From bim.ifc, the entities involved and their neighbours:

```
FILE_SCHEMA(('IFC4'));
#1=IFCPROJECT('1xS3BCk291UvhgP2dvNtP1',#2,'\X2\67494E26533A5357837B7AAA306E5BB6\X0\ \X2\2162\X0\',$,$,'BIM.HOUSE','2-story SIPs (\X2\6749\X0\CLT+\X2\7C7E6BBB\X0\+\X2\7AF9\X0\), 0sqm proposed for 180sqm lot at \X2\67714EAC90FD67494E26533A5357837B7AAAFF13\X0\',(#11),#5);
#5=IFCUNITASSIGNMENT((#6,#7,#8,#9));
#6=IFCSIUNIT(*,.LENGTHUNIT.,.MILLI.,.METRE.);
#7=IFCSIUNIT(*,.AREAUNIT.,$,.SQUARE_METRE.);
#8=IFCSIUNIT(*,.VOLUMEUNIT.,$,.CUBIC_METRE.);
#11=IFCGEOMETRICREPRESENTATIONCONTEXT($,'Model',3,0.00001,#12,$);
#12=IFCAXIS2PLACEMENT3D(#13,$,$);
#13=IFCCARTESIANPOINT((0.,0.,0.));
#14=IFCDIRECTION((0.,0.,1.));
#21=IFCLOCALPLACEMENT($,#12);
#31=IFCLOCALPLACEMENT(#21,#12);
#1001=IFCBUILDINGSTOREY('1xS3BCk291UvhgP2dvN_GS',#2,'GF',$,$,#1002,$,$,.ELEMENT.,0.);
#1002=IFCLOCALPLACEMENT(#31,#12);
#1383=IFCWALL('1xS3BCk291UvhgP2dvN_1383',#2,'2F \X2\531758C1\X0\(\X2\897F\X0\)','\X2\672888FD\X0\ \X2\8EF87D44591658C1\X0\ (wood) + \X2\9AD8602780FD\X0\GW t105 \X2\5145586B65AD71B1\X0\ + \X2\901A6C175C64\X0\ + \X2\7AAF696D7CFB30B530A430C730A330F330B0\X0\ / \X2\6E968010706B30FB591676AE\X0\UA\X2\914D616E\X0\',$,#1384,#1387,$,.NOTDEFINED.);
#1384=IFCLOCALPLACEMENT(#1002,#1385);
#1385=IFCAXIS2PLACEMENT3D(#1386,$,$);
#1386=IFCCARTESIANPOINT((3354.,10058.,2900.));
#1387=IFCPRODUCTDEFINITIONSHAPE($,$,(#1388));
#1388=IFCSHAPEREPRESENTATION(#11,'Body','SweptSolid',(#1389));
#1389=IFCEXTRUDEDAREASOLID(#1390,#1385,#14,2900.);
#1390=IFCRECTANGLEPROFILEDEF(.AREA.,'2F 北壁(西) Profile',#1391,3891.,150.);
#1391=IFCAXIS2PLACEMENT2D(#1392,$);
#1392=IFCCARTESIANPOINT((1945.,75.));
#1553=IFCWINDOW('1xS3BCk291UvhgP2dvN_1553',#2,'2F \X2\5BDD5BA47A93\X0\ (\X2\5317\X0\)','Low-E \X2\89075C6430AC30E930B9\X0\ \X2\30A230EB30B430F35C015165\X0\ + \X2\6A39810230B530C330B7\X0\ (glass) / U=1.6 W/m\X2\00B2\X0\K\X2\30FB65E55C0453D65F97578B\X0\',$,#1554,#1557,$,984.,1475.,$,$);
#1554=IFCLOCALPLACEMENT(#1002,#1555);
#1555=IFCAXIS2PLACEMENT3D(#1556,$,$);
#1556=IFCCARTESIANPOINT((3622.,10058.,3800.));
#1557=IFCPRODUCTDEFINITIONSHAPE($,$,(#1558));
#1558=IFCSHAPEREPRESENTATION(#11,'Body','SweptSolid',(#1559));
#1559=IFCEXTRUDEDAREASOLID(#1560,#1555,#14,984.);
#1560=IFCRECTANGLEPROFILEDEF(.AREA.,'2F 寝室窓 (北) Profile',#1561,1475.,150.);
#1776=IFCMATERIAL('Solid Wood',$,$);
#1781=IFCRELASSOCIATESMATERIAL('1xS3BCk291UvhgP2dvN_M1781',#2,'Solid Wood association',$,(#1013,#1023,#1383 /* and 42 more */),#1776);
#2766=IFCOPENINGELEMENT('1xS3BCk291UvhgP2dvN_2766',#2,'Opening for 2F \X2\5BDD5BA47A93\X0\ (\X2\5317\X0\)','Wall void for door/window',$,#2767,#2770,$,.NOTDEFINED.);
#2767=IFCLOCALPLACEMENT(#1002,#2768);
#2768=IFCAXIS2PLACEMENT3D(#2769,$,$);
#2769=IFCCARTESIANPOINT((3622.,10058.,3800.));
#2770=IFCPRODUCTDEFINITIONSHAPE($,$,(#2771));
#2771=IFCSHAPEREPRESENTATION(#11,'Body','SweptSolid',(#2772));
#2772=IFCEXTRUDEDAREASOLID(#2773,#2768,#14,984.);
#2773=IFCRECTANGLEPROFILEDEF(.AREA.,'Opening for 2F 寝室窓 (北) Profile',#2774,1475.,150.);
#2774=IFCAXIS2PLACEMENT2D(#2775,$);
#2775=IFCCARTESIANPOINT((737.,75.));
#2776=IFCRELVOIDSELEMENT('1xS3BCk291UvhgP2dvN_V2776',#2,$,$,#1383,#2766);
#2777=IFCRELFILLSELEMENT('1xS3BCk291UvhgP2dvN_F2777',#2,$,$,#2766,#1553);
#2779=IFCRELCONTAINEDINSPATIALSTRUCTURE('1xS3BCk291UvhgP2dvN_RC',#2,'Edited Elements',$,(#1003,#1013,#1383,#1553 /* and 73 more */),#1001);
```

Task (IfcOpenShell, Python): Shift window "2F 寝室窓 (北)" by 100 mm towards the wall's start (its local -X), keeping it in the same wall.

```python
import ifcopenshell
import ifcopenshell.api.geometry
import ifcopenshell.util.placement
import ifcopenshell.util.unit

model = ifcopenshell.open("bim.ifc")
unit_scale = ifcopenshell.util.unit.calculate_unit_scale(model)

window = model.by_guid("1xS3BCk291UvhgP2dvN_1553")
opening = window.FillsVoids[0].RelatingOpeningElement
wall = opening.VoidsElements[0].RelatingBuildingElement

wall_matrix = ifcopenshell.util.placement.get_local_placement(wall.ObjectPlacement)
shift = wall_matrix[:3, 0] * -0.1 / unit_scale
before = ifcopenshell.util.placement.get_local_placement(window.ObjectPlacement)[:3, 3].copy()

# The window is not placed relative to its opening, so move both.
for product in (opening, window):
    matrix = ifcopenshell.util.placement.get_local_placement(product.ObjectPlacement)
    matrix[:3, 3] += shift
    ifcopenshell.api.geometry.edit_object_placement(model, product=product, matrix=matrix, is_si=False)

after = ifcopenshell.util.placement.get_local_placement(window.ObjectPlacement)[:3, 3]
print("window moved by", (after - before).round(3) + 0.0)

model.write("bim_edited.ifc")
```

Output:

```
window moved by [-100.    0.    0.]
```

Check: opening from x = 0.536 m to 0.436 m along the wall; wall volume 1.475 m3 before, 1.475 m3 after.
